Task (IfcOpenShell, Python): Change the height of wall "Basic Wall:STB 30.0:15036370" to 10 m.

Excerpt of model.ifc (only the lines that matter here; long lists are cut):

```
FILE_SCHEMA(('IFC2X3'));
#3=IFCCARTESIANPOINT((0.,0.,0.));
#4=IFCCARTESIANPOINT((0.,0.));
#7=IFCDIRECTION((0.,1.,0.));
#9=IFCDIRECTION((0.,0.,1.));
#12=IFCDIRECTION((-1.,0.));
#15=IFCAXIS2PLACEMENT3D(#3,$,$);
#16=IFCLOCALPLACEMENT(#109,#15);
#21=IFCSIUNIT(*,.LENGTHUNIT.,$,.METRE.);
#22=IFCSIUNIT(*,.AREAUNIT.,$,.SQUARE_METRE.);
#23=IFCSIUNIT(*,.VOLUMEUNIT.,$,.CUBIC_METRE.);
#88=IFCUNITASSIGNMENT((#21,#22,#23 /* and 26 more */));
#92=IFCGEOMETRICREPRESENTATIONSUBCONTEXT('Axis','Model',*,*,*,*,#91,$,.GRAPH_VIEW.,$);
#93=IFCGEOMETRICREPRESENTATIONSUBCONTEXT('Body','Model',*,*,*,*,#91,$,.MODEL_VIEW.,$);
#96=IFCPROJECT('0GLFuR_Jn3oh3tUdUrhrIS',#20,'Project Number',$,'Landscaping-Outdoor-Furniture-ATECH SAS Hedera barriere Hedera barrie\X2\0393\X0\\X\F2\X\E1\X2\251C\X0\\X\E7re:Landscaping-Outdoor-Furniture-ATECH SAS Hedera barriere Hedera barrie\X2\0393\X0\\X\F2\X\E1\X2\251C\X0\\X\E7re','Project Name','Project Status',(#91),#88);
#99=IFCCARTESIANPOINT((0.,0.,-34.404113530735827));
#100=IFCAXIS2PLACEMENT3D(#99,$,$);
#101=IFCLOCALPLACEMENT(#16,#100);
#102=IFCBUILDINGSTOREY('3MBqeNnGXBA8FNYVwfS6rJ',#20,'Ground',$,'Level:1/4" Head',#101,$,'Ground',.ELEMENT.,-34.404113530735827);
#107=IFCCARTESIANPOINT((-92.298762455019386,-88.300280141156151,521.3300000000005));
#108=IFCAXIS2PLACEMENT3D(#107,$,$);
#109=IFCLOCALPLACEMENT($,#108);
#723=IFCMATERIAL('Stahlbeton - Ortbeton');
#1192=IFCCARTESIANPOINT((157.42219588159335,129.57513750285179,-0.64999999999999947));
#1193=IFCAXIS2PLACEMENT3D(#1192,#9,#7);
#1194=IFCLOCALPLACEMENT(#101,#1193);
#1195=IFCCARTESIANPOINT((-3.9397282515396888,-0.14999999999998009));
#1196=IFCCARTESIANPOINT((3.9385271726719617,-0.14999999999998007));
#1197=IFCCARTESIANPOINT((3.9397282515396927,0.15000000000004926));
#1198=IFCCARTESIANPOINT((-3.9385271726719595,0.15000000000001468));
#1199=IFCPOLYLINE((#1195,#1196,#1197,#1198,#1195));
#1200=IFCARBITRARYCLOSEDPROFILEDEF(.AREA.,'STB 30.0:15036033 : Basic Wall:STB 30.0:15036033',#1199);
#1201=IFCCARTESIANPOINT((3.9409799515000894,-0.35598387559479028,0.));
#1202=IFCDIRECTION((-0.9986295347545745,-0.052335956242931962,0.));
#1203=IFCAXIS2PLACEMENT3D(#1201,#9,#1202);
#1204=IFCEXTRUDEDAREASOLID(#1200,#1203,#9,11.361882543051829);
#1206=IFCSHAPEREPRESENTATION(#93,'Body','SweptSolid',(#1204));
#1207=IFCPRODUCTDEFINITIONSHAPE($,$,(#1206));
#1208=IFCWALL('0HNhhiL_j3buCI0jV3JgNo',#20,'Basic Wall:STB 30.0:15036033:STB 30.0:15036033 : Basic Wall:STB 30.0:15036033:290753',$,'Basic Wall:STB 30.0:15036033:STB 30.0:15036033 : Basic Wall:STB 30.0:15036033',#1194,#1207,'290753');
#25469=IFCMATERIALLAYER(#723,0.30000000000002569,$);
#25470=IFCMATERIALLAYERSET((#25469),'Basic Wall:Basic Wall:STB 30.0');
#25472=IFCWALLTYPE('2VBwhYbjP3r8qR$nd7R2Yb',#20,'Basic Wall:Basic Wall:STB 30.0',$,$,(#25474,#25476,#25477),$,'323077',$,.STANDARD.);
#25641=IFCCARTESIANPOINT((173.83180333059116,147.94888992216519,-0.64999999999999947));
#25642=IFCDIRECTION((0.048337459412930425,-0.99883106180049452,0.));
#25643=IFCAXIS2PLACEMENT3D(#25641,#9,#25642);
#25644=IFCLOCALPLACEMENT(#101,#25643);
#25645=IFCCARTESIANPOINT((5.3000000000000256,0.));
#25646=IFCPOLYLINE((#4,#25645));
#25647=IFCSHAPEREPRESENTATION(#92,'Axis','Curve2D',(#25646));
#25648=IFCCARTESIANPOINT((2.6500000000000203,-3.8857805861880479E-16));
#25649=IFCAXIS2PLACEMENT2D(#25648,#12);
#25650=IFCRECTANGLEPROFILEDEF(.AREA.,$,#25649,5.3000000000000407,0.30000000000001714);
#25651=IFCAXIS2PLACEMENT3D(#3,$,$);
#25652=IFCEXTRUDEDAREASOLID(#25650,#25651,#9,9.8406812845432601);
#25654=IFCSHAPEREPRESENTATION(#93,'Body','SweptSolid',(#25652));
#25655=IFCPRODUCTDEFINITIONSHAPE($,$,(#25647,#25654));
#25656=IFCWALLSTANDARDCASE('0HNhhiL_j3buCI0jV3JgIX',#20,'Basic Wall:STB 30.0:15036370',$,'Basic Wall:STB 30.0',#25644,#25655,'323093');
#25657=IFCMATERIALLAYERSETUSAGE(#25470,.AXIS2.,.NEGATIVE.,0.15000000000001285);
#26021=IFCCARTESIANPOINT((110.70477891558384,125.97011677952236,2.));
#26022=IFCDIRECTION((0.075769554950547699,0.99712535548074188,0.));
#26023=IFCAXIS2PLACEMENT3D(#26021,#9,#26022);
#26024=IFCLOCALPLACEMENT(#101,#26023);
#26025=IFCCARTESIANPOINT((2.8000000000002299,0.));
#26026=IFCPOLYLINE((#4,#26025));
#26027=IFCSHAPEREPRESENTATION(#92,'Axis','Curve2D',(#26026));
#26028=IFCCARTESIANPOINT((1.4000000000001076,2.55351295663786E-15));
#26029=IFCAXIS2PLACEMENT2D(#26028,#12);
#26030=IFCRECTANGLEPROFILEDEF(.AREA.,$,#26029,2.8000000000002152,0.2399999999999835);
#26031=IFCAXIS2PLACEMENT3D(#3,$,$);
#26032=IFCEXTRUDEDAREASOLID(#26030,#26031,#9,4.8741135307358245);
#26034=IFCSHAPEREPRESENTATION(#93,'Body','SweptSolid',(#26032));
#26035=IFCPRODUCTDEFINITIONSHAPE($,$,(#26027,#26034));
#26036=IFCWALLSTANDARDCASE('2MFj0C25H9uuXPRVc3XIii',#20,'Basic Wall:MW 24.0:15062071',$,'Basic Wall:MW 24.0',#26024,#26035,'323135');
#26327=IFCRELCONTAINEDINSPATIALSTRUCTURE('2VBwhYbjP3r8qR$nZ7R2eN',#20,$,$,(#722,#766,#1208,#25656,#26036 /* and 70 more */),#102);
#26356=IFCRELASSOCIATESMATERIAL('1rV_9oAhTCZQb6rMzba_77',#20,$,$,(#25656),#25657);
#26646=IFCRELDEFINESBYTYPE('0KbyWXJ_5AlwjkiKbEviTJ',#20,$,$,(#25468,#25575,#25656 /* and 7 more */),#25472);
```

```python
import ifcopenshell
import ifcopenshell.geom
import ifcopenshell.util.representation
import ifcopenshell.util.shape
import ifcopenshell.util.unit

model = ifcopenshell.open("model.ifc")
unit_scale = ifcopenshell.util.unit.calculate_unit_scale(model)
settings = ifcopenshell.geom.settings()


def volume(element):
    """Net volume in cubic metres, openings subtracted."""
    shape = ifcopenshell.geom.create_shape(settings, element)
    return ifcopenshell.util.shape.get_volume(shape.geometry)


wall = model.by_id(25656)
before = volume(wall)

body = ifcopenshell.util.representation.get_representation(wall, "Model", "Body")
solid = body.Items[0]
old_height = solid.Depth
solid.Depth = 10 / unit_scale
after = volume(wall)

print(f"height {old_height:g} -> {solid.Depth:g}, volume {before:.3f} -> {after:.3f} m3")

model.write("model_updated.ifc")
```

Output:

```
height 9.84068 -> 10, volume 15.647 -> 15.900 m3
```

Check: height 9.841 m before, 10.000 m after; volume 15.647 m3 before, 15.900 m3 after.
